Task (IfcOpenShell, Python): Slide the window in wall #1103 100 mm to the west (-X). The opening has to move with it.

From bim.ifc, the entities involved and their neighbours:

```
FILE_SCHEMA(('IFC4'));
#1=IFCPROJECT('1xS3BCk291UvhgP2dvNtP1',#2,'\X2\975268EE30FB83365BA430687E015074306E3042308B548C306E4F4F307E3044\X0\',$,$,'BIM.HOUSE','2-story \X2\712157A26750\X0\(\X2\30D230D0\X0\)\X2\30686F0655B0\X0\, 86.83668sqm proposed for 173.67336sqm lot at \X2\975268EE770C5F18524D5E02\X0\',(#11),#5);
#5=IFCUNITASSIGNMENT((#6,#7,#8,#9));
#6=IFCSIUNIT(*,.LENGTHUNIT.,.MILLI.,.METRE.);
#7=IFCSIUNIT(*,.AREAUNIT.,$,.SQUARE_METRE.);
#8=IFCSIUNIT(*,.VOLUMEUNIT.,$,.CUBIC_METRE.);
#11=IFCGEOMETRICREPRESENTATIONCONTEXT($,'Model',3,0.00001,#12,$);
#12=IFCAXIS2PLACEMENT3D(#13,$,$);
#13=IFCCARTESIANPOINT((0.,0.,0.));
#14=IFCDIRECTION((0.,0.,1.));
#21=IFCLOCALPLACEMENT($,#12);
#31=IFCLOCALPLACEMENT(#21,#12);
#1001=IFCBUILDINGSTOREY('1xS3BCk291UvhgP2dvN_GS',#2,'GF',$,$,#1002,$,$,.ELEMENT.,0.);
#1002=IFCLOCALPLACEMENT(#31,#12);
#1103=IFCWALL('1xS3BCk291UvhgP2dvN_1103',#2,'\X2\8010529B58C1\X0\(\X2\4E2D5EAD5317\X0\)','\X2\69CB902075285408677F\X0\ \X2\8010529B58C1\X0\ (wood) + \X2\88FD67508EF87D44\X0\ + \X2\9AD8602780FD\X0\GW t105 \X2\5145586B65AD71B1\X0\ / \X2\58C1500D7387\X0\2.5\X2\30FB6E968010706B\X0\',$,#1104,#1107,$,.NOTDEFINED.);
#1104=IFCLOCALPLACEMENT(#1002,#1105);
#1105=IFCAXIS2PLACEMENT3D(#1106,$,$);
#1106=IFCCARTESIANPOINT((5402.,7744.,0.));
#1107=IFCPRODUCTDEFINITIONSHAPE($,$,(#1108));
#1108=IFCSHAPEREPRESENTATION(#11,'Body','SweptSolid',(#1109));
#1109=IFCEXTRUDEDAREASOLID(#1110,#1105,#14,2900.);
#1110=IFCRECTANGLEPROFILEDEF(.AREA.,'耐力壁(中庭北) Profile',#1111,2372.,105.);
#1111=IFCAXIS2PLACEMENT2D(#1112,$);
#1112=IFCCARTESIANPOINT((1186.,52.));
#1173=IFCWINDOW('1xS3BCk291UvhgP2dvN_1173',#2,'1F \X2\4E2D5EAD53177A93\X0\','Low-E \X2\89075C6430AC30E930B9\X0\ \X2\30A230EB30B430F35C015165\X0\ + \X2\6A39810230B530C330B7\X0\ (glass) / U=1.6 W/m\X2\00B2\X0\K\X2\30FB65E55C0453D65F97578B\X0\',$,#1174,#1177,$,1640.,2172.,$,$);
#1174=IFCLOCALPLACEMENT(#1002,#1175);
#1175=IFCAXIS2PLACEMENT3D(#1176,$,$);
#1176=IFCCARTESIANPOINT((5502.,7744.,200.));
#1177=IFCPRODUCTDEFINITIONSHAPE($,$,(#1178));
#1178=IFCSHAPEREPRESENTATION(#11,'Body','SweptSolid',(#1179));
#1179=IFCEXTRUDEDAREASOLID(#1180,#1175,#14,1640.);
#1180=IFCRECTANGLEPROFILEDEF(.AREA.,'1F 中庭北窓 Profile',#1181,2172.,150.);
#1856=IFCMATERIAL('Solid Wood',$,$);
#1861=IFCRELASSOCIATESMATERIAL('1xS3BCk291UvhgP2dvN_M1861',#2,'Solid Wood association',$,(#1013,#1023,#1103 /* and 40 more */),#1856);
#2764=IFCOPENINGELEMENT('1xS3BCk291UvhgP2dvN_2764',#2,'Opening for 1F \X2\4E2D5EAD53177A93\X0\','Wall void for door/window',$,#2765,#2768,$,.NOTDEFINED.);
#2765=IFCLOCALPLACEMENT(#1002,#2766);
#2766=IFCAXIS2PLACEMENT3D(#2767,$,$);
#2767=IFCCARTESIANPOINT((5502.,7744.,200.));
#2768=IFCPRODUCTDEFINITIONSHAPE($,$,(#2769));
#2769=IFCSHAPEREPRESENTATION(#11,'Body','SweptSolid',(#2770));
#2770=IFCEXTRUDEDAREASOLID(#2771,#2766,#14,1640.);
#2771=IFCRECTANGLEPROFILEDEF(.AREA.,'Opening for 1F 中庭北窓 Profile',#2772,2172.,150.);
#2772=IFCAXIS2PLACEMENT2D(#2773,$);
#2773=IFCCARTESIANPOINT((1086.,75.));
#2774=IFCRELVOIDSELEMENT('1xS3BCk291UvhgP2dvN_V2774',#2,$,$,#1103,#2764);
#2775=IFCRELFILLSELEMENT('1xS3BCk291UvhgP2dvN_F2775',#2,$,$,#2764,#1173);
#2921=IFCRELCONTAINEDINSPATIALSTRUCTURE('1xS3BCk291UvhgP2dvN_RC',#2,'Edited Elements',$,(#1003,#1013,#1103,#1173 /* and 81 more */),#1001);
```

```python
import ifcopenshell
import ifcopenshell.api.geometry
import ifcopenshell.util.placement

model = ifcopenshell.open("bim.ifc")

window = model.by_guid("1xS3BCk291UvhgP2dvN_1173")
opening = window.FillsVoids[0].RelatingOpeningElement
wall = opening.VoidsElements[0].RelatingBuildingElement

wall_matrix = ifcopenshell.util.placement.get_local_placement(wall.ObjectPlacement)
shift = wall_matrix[:3, 0] * -100.0
before = ifcopenshell.util.placement.get_local_placement(window.ObjectPlacement)[:3, 3].copy()

# The window is not placed relative to its opening, so move both.
for product in (opening, window):
    matrix = ifcopenshell.util.placement.get_local_placement(product.ObjectPlacement)
    matrix[:3, 3] += shift
    ifcopenshell.api.geometry.edit_object_placement(model, product=product, matrix=matrix, is_si=False)

after = ifcopenshell.util.placement.get_local_placement(window.ObjectPlacement)[:3, 3]
print("window moved by", (after - before).round(3) + 0.0)

model.write("bim_rev.ifc")
```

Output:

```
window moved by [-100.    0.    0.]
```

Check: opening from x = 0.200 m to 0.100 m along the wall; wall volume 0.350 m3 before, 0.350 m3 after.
